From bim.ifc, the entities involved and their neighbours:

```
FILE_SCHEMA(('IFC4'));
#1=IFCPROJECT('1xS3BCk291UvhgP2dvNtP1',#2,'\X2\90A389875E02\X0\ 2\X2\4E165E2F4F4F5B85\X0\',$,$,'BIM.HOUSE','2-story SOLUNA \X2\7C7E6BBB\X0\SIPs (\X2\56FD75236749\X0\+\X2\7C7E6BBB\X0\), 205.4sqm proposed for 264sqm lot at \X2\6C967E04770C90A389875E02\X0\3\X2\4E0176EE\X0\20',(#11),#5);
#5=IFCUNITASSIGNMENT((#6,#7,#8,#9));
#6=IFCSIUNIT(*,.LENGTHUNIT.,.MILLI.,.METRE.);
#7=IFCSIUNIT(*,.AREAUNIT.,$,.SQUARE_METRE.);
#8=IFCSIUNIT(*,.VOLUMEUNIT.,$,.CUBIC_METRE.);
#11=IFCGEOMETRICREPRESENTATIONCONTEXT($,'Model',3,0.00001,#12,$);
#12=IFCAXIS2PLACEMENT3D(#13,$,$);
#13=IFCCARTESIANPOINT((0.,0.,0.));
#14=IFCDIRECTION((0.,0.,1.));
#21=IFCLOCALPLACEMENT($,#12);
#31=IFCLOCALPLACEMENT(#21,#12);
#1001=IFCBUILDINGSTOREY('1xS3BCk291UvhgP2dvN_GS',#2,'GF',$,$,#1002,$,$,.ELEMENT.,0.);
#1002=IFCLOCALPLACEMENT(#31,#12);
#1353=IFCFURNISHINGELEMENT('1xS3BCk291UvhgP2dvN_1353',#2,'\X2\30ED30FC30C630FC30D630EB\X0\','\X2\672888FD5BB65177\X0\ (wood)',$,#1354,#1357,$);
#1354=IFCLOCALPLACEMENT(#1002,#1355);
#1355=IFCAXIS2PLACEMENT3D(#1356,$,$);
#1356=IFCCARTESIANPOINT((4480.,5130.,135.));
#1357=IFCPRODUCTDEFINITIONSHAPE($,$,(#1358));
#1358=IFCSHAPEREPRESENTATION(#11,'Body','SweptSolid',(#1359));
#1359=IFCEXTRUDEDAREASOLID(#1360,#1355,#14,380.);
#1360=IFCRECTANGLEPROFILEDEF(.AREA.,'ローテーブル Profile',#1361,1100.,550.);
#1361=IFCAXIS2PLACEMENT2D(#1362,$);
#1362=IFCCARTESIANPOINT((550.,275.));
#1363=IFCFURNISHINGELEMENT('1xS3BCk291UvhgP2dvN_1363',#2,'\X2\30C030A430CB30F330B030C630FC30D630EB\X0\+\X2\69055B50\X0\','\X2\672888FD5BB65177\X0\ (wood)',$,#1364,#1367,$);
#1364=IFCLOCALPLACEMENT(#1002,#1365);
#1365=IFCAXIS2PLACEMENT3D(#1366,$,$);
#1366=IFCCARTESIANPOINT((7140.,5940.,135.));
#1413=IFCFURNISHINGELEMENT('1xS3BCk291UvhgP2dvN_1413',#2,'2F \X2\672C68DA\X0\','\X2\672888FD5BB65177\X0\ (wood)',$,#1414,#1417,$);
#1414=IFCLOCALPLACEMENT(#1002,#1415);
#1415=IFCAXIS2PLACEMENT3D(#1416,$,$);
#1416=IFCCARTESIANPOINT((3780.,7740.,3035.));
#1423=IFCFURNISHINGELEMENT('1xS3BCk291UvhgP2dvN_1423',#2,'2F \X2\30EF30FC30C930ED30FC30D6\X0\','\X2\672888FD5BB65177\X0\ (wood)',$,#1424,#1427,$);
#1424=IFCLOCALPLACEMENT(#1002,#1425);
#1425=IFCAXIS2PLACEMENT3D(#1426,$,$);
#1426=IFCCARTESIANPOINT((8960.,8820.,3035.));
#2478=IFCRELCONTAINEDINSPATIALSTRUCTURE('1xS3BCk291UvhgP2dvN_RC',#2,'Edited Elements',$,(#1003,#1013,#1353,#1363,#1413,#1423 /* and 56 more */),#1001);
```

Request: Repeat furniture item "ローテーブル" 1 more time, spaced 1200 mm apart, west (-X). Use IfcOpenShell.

```python
import numpy as np
import ifcopenshell
import ifcopenshell.api.geometry
import ifcopenshell.api.root
import ifcopenshell.util.element
import ifcopenshell.util.placement

model = ifcopenshell.open("bim.ifc")


def reuse_history(source, copy):
    """copy_class also copies each property set's owner history, people and application; keep the originals."""
    for rel in copy.IsDefinedBy:
        if rel.is_a("IfcRelDefinesByProperties") and (history := rel.RelatingPropertyDefinition.OwnerHistory):
            rel.RelatingPropertyDefinition.OwnerHistory = source.OwnerHistory
            ifcopenshell.util.element.remove_deep2(model, history)


source = model.by_guid("1xS3BCk291UvhgP2dvN_1353")
base = ifcopenshell.util.placement.get_local_placement(source.ObjectPlacement)
step = np.array([-1.0, 0.0, 0.0]) * 1200.0

for i in range(1, 2):
    copy = ifcopenshell.api.root.copy_class(model, product=source)
    copy.Representation = ifcopenshell.util.element.copy_deep(
        model, source.Representation, exclude=["IfcGeometricRepresentationContext", "IfcRepresentationMap"]
    )
    reuse_history(source, copy)
    matrix = base.copy()
    matrix[:3, 3] += i * step
    print("added at", matrix[:3, 3].round(3) + 0.0)
    ifcopenshell.api.geometry.edit_object_placement(model, product=copy, matrix=matrix, is_si=False)

model.write("bim-out.ifc")
```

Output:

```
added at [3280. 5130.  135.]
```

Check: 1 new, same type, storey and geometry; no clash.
